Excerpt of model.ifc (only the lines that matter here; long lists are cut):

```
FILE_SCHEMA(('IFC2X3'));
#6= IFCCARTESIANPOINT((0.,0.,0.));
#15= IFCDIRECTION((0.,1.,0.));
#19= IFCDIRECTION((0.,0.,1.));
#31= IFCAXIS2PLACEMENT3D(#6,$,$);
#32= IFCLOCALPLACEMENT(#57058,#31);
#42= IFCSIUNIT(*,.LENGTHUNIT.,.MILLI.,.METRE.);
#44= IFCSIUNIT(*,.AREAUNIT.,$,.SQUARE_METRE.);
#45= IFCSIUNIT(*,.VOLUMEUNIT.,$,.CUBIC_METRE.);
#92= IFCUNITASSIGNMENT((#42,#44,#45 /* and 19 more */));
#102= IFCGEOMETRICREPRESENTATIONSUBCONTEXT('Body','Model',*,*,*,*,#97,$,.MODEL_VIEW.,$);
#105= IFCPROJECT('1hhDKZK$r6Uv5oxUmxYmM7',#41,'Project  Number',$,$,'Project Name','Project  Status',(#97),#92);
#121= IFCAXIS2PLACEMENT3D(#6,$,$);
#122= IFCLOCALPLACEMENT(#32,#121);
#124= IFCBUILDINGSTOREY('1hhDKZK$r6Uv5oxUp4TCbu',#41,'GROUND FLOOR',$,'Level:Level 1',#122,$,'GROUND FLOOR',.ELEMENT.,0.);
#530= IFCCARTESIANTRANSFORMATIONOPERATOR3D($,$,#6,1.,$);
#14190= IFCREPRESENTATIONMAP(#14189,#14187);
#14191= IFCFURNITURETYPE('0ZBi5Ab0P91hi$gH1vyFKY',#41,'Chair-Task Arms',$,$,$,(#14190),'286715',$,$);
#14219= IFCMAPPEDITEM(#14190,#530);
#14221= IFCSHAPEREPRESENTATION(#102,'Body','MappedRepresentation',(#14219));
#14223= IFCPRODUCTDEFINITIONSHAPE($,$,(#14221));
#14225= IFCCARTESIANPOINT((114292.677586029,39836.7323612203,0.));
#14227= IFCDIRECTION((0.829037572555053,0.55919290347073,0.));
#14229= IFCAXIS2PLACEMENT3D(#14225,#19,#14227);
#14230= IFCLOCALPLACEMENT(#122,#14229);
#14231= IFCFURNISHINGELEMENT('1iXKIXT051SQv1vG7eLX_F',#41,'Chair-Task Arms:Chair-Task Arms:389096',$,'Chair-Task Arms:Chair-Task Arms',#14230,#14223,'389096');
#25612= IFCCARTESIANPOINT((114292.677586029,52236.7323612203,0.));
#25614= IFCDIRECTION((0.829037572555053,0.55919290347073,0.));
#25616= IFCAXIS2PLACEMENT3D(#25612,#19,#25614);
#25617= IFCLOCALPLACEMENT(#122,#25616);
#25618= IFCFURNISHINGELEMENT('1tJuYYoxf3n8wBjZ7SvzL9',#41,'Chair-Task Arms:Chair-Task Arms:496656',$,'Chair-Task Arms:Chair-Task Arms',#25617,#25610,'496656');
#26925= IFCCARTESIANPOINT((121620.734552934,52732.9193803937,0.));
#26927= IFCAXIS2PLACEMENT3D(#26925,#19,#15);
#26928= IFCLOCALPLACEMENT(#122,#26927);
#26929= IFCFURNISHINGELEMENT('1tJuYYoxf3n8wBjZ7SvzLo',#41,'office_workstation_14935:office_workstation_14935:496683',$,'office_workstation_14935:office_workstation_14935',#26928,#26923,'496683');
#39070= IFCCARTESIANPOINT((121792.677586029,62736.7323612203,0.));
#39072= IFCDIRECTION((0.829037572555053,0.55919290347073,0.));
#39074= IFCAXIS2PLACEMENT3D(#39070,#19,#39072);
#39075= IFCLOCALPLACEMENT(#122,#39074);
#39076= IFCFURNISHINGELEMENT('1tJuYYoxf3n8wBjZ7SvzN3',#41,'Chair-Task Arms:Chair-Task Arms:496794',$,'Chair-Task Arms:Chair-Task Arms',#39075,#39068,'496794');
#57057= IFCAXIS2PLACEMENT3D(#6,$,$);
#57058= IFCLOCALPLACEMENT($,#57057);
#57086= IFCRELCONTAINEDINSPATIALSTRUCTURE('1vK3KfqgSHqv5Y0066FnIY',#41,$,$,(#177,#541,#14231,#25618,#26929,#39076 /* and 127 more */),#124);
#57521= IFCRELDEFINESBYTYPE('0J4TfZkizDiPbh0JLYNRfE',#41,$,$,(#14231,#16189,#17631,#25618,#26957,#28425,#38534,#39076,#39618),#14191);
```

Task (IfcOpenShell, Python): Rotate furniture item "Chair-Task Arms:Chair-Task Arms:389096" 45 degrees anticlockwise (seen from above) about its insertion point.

```python
import ifcopenshell
import ifcopenshell.api.geometry
import ifcopenshell.util.placement

model = ifcopenshell.open("model.ifc")

item = model.by_guid("1iXKIXT051SQv1vG7eLX_F")
matrix = ifcopenshell.util.placement.get_local_placement(item.ObjectPlacement)
matrix = matrix @ ifcopenshell.util.placement.rotation(45, "Z")
ifcopenshell.api.geometry.edit_object_placement(model, product=item, matrix=matrix, is_si=False)

print(ifcopenshell.util.placement.get_local_placement(item.ObjectPlacement).round(3) + 0.0)

model.write("model_v2.ifc")
```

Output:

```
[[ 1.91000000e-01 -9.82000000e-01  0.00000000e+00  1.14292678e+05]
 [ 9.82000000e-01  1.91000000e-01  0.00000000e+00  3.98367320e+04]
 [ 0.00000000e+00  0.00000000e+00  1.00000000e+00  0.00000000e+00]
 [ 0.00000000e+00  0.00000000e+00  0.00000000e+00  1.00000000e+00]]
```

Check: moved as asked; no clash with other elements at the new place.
